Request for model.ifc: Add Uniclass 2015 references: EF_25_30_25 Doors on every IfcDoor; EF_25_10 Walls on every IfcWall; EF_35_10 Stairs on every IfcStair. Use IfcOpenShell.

First a look at what the model holds.

```python
import ifcopenshell

model = ifcopenshell.open("model.ifc")
print(model.schema)
print("classifications:", [c.Name for c in model.by_type("IfcClassification")])
for ifc_class in ("IfcDoor", "IfcRoof", "IfcStair", "IfcWall", "IfcWindow"):
    print(ifc_class, len(model.by_type(ifc_class)))
```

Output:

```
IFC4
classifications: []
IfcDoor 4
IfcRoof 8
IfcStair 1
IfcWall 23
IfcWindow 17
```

```python
import ifcopenshell
import ifcopenshell.api.classification

model = ifcopenshell.open("model.ifc")

system = ifcopenshell.api.classification.add_classification(model, classification="Uniclass 2015")

codes = {
    "IfcDoor": ("EF_25_30_25", "Doors"),
    "IfcWall": ("EF_25_10", "Walls"),
    "IfcStair": ("EF_35_10", "Stairs"),
}
for ifc_class, (code, name) in codes.items():
    products = model.by_type(ifc_class)
    ifcopenshell.api.classification.add_reference(
        model, products=products, classification=system, identification=code, name=name
    )
    print(code, len(products))

model.write("model_edited.ifc")
```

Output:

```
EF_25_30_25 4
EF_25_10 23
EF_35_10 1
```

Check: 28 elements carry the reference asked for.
